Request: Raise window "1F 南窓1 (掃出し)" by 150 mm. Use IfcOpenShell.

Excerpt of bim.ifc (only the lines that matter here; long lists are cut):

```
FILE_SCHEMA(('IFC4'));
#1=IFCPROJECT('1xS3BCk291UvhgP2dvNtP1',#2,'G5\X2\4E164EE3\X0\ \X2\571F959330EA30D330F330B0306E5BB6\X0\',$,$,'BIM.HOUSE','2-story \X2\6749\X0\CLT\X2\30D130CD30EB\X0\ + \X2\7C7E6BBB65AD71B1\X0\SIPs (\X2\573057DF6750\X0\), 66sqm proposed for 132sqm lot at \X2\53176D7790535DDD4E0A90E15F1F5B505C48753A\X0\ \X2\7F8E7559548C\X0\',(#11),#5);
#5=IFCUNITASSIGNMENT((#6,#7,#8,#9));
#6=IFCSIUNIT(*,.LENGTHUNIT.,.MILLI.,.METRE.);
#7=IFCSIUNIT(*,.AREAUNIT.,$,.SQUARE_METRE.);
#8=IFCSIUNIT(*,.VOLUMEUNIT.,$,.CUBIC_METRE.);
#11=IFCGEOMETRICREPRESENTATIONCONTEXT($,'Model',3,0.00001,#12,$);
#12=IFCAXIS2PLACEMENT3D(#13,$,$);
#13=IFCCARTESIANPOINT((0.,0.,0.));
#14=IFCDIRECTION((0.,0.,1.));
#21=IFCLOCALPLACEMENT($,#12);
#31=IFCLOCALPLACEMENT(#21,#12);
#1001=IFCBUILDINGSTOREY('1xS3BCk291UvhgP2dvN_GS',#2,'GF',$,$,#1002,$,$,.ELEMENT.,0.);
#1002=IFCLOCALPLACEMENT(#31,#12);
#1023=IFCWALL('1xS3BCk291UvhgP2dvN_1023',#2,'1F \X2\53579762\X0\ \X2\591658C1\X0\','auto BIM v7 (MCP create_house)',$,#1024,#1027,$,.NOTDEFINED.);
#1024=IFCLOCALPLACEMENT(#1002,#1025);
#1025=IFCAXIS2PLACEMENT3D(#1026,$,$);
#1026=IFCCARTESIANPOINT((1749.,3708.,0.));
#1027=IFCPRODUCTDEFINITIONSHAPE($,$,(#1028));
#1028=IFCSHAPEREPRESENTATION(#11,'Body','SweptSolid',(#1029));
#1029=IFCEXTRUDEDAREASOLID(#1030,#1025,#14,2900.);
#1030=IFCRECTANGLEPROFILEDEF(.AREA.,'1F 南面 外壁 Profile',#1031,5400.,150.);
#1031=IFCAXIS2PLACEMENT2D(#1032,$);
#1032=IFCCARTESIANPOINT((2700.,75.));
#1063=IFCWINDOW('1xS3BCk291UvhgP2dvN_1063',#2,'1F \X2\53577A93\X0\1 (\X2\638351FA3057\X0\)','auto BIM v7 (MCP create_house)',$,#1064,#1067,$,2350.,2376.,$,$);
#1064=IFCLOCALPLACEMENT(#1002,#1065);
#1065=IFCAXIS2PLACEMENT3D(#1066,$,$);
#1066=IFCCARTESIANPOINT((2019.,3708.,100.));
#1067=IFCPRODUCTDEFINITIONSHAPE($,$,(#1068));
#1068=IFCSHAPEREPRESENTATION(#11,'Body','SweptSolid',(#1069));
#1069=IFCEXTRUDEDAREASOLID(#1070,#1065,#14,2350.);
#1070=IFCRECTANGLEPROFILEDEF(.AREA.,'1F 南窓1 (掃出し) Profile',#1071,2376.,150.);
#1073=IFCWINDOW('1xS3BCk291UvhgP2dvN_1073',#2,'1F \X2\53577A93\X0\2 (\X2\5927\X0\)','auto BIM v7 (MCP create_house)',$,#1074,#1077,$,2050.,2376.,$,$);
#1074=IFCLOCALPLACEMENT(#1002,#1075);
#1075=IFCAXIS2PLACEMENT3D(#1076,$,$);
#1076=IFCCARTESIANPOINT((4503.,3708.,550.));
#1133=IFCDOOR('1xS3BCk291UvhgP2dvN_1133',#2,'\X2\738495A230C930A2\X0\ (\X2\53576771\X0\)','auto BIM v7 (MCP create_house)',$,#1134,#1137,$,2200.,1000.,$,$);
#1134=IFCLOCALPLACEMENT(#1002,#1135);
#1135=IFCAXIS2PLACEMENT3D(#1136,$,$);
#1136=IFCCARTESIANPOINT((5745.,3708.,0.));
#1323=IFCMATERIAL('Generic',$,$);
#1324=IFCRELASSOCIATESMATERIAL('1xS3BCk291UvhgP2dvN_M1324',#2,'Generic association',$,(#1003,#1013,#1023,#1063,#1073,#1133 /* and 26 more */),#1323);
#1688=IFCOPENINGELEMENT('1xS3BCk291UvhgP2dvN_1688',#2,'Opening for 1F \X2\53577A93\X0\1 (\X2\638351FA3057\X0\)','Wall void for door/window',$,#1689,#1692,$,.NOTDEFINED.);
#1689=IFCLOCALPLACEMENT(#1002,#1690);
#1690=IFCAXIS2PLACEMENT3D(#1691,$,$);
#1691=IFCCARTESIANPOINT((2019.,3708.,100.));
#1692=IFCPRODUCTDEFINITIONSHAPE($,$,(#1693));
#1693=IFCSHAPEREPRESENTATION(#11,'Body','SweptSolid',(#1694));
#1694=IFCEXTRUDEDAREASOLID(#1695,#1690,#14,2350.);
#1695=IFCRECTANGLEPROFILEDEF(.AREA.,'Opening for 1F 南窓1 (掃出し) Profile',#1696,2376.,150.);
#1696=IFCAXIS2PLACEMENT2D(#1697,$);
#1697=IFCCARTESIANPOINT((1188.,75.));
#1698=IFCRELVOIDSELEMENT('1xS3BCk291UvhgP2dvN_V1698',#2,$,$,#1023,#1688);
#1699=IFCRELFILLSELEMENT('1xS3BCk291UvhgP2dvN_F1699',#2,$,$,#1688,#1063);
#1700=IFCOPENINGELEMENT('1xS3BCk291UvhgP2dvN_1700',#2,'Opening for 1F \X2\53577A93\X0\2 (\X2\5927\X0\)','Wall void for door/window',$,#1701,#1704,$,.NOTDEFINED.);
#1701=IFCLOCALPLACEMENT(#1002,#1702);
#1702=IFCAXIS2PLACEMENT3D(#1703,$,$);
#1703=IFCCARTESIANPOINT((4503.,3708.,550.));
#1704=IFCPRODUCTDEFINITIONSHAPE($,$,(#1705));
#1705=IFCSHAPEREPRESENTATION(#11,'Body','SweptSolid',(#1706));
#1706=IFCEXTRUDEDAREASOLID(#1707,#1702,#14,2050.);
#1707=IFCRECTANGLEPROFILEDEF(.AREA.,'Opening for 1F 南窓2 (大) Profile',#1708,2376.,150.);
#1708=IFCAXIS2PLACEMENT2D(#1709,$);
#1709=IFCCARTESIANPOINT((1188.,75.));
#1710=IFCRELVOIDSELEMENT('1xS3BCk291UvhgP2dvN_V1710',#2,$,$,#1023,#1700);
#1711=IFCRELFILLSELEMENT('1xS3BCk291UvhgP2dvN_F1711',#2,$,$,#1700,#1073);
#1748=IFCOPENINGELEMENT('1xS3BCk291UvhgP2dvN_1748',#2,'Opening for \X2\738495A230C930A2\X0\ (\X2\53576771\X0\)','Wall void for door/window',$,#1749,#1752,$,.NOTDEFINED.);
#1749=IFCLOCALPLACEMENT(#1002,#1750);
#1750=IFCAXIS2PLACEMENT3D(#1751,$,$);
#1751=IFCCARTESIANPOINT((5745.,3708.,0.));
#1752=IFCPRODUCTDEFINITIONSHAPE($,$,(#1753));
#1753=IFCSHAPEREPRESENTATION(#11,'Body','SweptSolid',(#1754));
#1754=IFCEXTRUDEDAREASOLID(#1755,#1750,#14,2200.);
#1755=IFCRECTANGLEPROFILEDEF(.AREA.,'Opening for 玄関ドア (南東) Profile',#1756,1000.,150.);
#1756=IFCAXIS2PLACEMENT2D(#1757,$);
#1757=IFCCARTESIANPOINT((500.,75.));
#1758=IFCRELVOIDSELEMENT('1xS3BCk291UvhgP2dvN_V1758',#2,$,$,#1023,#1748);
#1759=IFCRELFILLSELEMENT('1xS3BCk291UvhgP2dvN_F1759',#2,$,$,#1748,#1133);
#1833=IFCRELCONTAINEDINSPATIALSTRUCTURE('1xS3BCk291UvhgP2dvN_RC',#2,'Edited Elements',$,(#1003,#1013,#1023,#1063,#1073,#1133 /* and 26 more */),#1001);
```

```python
import numpy as np
import ifcopenshell
import ifcopenshell.api.geometry
import ifcopenshell.util.placement
import ifcopenshell.util.unit

model = ifcopenshell.open("bim.ifc")
unit_scale = ifcopenshell.util.unit.calculate_unit_scale(model)

window = model.by_guid("1xS3BCk291UvhgP2dvN_1063")
opening = window.FillsVoids[0].RelatingOpeningElement
dz = 0.15 / unit_scale

shift = np.array([0.0, 0.0, dz])
# The window is not placed relative to its opening, so move both.
for product in (opening, window):
    matrix = ifcopenshell.util.placement.get_local_placement(product.ObjectPlacement)
    matrix[:3, 3] += shift
    ifcopenshell.api.geometry.edit_object_placement(model, product=product, matrix=matrix, is_si=False)

print(f"moved by {dz * unit_scale:+.3f} m")

model.write("bim-out.ifc")
```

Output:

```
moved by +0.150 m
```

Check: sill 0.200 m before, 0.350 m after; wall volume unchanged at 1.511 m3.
